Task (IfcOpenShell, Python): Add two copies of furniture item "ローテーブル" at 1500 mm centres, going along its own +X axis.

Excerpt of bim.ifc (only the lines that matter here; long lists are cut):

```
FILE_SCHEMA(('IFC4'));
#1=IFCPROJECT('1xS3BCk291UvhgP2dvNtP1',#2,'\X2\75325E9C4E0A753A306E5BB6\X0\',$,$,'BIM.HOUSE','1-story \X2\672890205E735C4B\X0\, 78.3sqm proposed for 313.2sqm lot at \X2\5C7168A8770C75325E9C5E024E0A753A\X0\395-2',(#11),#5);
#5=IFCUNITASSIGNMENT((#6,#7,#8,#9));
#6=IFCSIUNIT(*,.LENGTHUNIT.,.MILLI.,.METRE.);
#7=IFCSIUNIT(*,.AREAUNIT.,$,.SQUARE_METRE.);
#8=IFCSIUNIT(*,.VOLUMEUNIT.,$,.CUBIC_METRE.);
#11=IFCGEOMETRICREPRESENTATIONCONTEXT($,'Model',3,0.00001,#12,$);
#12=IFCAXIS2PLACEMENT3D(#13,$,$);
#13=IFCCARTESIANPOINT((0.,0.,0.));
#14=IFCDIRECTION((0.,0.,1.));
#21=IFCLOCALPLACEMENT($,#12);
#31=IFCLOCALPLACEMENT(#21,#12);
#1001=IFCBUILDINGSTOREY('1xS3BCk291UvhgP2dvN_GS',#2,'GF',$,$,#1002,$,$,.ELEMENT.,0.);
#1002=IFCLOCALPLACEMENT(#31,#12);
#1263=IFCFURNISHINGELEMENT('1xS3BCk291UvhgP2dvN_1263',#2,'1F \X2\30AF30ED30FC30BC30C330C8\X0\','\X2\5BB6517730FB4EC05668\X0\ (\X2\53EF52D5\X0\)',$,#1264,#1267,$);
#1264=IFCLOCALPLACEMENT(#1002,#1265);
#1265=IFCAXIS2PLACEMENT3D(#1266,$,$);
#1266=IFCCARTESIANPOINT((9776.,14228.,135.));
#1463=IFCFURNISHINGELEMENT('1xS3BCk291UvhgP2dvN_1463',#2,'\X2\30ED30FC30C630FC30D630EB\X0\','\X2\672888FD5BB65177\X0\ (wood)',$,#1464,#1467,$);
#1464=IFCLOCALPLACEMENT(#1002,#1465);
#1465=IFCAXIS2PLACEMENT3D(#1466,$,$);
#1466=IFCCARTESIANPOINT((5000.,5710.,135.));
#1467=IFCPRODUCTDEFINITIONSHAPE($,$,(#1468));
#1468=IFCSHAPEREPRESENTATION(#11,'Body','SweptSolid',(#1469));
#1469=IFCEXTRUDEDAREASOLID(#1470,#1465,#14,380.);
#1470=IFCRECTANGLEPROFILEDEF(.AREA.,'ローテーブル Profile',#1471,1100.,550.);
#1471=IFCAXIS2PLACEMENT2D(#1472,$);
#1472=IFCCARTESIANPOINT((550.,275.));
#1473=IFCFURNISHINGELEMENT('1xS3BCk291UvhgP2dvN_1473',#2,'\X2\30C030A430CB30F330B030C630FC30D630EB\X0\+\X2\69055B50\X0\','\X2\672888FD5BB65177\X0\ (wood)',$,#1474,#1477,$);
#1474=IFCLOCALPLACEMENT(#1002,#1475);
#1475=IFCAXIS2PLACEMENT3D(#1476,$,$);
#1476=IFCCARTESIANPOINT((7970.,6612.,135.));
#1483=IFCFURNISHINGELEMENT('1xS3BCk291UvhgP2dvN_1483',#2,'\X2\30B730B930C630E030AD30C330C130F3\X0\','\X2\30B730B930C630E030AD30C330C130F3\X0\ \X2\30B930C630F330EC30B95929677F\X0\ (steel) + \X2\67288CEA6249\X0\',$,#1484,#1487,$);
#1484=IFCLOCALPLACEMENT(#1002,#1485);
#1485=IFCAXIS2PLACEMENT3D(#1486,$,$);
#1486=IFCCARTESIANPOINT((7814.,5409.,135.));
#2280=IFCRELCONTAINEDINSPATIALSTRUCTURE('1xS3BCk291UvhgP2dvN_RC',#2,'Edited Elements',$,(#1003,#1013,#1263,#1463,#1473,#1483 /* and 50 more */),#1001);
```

```python
import ifcopenshell
import ifcopenshell.api.geometry
import ifcopenshell.api.root
import ifcopenshell.util.element
import ifcopenshell.util.placement
import ifcopenshell.util.unit

model = ifcopenshell.open("bim.ifc")
unit_scale = ifcopenshell.util.unit.calculate_unit_scale(model)


def reuse_history(source, copy):
    """copy_class also copies each property set's owner history, people and application; keep the originals."""
    for rel in copy.IsDefinedBy:
        if rel.is_a("IfcRelDefinesByProperties") and (history := rel.RelatingPropertyDefinition.OwnerHistory):
            rel.RelatingPropertyDefinition.OwnerHistory = source.OwnerHistory
            ifcopenshell.util.element.remove_deep2(model, history)


source = model.by_guid("1xS3BCk291UvhgP2dvN_1463")
base = ifcopenshell.util.placement.get_local_placement(source.ObjectPlacement)
step = base[:3, 0] * 1.5 / unit_scale

for i in range(1, 3):
    copy = ifcopenshell.api.root.copy_class(model, product=source)
    copy.Representation = ifcopenshell.util.element.copy_deep(
        model, source.Representation, exclude=["IfcGeometricRepresentationContext", "IfcRepresentationMap"]
    )
    reuse_history(source, copy)
    matrix = base.copy()
    matrix[:3, 3] += i * step
    print("added at", matrix[:3, 3].round(3) + 0.0)
    ifcopenshell.api.geometry.edit_object_placement(model, product=copy, matrix=matrix, is_si=False)

model.write("bim_rev.ifc")
```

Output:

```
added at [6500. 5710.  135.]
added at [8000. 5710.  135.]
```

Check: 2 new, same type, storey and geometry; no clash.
